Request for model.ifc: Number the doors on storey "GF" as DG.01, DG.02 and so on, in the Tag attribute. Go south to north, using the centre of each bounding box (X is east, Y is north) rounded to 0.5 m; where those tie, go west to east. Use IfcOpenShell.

First a look at what the model holds.

```python
import ifcopenshell
import ifcopenshell.util.element
import ifcopenshell.util.placement

model = ifcopenshell.open("model.ifc")
print(model.schema)
storey = next(s for s in model.by_type("IfcBuildingStorey") if s.Name == "GF")
doors = [e for e in ifcopenshell.util.element.get_decomposition(storey) if e.is_a("IfcDoor")]
for e in sorted(doors, key=lambda e: e.id()):
    origin = ifcopenshell.util.placement.get_local_placement(e.ObjectPlacement)[:3, 3]
    print(e.id(), e.Tag, e.Name, origin.round(2) + 0.0, sep=" | ")
```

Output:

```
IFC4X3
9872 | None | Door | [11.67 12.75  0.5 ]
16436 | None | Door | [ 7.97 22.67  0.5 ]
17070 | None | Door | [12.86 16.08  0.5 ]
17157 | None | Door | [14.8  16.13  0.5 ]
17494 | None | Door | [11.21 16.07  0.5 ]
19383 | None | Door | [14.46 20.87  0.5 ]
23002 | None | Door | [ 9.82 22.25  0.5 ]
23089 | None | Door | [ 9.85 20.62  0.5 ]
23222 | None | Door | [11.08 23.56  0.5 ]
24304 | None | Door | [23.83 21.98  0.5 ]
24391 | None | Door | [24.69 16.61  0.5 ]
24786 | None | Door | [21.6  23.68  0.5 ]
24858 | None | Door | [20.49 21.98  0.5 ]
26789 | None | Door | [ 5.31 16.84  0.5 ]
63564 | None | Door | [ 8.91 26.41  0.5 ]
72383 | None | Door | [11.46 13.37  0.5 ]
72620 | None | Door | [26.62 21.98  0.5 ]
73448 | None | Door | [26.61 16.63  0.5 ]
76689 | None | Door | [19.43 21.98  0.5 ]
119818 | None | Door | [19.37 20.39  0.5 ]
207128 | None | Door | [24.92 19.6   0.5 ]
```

```python
import ifcopenshell
import ifcopenshell.geom
import ifcopenshell.util.element
import ifcopenshell.util.shape

model = ifcopenshell.open("model.ifc")
settings = ifcopenshell.geom.settings()
settings.set("use-world-coords", True)


def centre(element):
    shape = ifcopenshell.geom.create_shape(settings, element)
    return ifcopenshell.util.shape.get_bbox_centroid(shape.geometry)


storey = next(s for s in model.by_type("IfcBuildingStorey") if s.Name == "GF")
doors = [e for e in ifcopenshell.util.element.get_decomposition(storey) if e.is_a("IfcDoor")]

# Insertion points can sit at a corner or the storey origin, so sort by the geometry (in metres).
centres = {e: centre(e) for e in doors}
doors.sort(key=lambda e: (round(centres[e][1] / 0.5), centres[e][0]))

for i, e in enumerate(doors, start=1):
    number = f"DG.{i:02d}"
    e.Tag = number
    print(e.id(), number)

model.write("model_rev.ifc")
```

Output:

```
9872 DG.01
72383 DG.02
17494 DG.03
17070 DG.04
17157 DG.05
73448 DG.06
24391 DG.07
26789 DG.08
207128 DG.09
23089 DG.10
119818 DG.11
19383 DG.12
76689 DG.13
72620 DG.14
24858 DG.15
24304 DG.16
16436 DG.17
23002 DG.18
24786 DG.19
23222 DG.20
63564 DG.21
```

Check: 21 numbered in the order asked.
